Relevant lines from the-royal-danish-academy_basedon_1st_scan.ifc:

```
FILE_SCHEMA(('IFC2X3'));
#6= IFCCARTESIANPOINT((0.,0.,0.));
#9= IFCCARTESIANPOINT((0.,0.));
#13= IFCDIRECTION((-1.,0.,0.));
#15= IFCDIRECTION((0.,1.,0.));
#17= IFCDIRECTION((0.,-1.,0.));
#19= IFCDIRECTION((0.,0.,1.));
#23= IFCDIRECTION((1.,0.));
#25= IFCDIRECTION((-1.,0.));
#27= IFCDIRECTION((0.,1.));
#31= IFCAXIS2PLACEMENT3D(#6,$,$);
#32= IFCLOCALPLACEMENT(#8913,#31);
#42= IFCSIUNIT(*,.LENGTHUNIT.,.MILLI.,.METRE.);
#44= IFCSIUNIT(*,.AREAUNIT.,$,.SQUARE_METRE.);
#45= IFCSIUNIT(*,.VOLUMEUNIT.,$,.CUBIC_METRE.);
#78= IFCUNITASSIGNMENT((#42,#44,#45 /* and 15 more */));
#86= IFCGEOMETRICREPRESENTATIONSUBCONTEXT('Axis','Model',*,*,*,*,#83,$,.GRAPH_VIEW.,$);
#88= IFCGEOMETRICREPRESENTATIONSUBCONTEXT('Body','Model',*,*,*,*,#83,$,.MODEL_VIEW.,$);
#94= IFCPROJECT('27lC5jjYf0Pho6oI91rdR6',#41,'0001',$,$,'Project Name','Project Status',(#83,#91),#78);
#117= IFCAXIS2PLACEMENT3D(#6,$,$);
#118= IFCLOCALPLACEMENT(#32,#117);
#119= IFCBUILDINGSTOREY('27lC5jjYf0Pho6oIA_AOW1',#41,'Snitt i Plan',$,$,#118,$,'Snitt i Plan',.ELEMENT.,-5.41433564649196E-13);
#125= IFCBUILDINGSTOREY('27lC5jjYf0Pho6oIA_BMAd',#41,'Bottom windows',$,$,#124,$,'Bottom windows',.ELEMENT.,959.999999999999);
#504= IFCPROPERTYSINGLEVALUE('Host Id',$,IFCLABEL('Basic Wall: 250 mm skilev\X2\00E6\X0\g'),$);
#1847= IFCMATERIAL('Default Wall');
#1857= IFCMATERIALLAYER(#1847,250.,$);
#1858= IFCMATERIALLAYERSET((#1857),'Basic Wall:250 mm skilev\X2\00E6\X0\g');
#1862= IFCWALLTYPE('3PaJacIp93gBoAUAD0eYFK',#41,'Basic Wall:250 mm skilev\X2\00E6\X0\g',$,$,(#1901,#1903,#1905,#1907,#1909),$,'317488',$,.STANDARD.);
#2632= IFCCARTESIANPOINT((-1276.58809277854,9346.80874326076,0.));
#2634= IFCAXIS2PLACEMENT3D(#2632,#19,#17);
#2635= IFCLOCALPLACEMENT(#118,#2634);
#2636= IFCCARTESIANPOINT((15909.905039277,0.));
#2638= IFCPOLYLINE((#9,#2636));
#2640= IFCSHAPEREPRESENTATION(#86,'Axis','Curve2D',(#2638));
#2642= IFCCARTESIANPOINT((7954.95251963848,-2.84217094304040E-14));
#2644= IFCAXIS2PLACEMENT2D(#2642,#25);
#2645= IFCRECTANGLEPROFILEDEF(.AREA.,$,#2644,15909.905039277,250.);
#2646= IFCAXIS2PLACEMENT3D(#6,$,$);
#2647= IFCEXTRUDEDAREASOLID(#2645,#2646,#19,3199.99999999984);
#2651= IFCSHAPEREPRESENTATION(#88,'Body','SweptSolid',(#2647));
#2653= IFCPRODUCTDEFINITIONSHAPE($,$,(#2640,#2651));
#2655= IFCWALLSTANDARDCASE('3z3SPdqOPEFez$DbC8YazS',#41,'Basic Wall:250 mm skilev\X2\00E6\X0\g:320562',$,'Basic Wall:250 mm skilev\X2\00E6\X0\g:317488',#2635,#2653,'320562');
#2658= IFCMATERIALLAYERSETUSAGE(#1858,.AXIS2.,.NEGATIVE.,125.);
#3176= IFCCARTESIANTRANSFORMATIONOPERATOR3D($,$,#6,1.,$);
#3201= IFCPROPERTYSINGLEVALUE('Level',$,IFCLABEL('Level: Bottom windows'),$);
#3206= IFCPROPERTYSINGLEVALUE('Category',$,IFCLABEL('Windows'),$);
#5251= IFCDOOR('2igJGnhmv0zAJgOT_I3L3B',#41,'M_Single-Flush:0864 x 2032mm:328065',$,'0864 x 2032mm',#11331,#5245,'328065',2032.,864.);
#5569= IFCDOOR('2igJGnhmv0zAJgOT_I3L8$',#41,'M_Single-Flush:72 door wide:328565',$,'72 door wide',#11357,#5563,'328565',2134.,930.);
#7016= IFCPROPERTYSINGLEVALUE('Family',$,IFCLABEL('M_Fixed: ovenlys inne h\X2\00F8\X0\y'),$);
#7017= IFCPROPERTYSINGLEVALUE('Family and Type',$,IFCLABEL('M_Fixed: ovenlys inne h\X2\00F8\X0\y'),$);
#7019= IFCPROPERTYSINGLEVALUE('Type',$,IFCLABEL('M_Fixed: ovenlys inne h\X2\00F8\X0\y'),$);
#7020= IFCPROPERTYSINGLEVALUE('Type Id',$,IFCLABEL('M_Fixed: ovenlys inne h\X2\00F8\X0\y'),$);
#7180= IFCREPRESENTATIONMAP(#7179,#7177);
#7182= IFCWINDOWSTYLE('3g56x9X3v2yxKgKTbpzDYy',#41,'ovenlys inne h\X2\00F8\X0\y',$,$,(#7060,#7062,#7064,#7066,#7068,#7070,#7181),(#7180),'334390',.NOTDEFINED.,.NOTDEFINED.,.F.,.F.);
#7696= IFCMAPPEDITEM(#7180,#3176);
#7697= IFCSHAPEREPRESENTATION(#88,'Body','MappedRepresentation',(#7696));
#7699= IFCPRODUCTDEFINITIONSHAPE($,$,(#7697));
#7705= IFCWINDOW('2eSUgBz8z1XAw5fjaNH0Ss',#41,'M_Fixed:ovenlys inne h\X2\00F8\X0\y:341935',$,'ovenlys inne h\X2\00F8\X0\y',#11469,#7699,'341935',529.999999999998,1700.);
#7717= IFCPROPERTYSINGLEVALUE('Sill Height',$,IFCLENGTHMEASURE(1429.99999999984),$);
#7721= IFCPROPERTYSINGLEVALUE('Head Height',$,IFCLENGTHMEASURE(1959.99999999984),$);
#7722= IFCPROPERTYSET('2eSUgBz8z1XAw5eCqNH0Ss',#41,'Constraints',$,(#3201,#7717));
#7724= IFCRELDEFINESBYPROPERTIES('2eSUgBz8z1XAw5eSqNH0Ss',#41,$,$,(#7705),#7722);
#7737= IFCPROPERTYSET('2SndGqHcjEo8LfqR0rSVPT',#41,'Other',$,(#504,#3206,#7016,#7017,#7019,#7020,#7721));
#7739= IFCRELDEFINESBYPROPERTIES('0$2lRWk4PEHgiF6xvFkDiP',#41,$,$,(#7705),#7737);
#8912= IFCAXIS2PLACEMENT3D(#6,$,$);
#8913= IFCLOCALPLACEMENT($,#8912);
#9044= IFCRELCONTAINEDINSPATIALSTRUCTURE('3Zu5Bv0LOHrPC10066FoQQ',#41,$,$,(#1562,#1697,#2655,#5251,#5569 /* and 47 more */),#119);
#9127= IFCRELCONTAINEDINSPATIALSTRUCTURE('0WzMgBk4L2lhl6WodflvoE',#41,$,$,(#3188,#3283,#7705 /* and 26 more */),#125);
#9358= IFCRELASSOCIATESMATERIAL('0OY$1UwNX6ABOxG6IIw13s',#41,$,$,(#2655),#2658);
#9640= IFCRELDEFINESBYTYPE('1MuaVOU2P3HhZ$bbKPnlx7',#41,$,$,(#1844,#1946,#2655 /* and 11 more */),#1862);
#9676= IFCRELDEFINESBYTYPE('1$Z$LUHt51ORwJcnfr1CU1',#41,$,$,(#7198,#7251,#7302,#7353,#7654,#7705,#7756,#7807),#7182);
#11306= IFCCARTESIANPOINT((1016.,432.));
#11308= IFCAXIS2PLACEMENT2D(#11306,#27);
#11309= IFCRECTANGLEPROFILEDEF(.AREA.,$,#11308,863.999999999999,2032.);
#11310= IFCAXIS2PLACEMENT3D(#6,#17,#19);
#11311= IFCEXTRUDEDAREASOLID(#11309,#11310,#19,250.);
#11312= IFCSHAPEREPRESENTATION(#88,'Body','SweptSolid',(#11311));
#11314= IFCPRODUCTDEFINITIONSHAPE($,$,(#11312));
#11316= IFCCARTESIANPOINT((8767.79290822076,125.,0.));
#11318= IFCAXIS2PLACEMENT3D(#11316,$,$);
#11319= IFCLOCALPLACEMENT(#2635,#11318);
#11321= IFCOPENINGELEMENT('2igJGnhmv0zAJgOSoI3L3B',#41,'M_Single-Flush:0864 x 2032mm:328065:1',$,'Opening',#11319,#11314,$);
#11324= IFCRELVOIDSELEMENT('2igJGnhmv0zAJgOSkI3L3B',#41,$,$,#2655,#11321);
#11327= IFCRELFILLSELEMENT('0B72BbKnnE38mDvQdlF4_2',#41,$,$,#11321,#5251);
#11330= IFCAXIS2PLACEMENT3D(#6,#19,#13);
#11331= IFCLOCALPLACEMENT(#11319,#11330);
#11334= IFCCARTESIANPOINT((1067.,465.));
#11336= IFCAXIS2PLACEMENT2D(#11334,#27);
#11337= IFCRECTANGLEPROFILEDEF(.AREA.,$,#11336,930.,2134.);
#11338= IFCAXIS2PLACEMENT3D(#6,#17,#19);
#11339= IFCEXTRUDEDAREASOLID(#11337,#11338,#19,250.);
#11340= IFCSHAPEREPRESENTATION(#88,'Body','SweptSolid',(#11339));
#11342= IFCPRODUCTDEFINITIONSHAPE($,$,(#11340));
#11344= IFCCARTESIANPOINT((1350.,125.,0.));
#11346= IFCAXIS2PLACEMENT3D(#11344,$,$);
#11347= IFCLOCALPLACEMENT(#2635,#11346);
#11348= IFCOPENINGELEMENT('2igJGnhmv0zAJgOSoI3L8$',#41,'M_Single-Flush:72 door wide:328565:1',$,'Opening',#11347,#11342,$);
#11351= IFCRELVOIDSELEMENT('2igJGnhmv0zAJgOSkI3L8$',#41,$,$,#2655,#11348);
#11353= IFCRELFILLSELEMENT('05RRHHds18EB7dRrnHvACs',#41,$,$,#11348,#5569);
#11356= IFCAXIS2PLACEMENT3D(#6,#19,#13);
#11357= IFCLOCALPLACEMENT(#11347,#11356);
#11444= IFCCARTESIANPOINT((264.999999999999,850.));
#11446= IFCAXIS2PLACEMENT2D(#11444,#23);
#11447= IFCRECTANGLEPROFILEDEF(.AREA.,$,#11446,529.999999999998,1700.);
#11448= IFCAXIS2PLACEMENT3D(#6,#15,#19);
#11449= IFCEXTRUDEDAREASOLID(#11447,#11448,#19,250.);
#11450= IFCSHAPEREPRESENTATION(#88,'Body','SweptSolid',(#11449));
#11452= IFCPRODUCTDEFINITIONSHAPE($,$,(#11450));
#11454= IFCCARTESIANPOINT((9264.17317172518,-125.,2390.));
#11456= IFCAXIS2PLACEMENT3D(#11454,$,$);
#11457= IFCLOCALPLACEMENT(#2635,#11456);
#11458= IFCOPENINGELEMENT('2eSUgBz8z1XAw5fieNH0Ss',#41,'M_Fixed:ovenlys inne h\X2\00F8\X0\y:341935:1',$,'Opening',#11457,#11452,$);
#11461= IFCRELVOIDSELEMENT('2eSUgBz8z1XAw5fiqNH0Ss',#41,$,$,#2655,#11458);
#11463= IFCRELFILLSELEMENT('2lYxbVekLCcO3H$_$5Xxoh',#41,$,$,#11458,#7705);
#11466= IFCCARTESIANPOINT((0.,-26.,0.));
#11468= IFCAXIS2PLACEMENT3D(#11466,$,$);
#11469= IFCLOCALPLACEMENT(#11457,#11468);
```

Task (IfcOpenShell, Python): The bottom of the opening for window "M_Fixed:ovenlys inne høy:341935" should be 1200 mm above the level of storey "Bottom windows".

```python
import numpy as np
import ifcopenshell
import ifcopenshell.api.geometry
import ifcopenshell.api.pset
import ifcopenshell.geom
import ifcopenshell.util.element
import ifcopenshell.util.placement
import ifcopenshell.util.shape
import ifcopenshell.util.unit

model = ifcopenshell.open("the-royal-danish-academy_basedon_1st_scan.ifc")
unit_scale = ifcopenshell.util.unit.calculate_unit_scale(model)

window = model.by_guid("2eSUgBz8z1XAw5fjaNH0Ss")
opening = window.FillsVoids[0].RelatingOpeningElement
storey = ifcopenshell.util.element.get_container(window, ifc_class="IfcBuildingStorey")
level = ifcopenshell.util.placement.get_local_placement(storey.ObjectPlacement)[2, 3]

# The opening's origin need not be at the sill, so measure its lowest point.
shape = ifcopenshell.geom.create_shape(ifcopenshell.geom.settings(), opening)
bottom = ifcopenshell.util.shape.get_shape_bottom_elevation(shape, shape.geometry) / unit_scale
dz = level + 1.2 / unit_scale - bottom

shift = np.array([0.0, 0.0, dz])
# The window is placed relative to its opening, so it follows when the opening moves.
matrix = ifcopenshell.util.placement.get_local_placement(opening.ObjectPlacement)
matrix[:3, 3] += shift
ifcopenshell.api.geometry.edit_object_placement(
    model, product=opening, matrix=matrix, is_si=False, should_transform_children=True
)

# Keep the stored heights in step.
pset = model.by_id(ifcopenshell.util.element.get_pset(window, "Constraints", should_inherit=False)["id"])
ifcopenshell.api.pset.edit_pset(model, pset=pset, properties={
    "Sill Height": model.create_entity("IfcLengthMeasure", ifcopenshell.util.element.get_pset(window, "Constraints", "Sill Height") + dz),
})
pset = model.by_id(ifcopenshell.util.element.get_pset(window, "Other", should_inherit=False)["id"])
ifcopenshell.api.pset.edit_pset(model, pset=pset, properties={
    "Head Height": model.create_entity("IfcLengthMeasure", ifcopenshell.util.element.get_pset(window, "Other", "Head Height") + dz),
})

print(f"moved by {dz * unit_scale:+.3f} m")

model.write("the-royal-danish-academy_basedon_1st_scan_rev.ifc")
```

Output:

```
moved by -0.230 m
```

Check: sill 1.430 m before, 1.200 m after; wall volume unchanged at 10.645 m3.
